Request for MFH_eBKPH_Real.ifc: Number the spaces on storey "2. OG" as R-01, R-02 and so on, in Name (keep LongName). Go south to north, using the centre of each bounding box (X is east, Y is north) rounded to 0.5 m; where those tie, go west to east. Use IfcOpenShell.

First a look at what the model holds.

```python
import ifcopenshell
import ifcopenshell.util.element
import ifcopenshell.util.placement

model = ifcopenshell.open("MFH_eBKPH_Real.ifc")
print(model.schema)
storey = next(s for s in model.by_type("IfcBuildingStorey") if s.Name == "2. OG")
spaces = [e for e in ifcopenshell.util.element.get_decomposition(storey) if e.is_a("IfcSpace")]
for e in sorted(spaces, key=lambda e: e.id()):
    origin = ifcopenshell.util.placement.get_local_placement(e.ObjectPlacement)[:3, 3]
    print(e.id(), e.Name, e.LongName, origin.round(2) + 0.0, sep=" | ")
```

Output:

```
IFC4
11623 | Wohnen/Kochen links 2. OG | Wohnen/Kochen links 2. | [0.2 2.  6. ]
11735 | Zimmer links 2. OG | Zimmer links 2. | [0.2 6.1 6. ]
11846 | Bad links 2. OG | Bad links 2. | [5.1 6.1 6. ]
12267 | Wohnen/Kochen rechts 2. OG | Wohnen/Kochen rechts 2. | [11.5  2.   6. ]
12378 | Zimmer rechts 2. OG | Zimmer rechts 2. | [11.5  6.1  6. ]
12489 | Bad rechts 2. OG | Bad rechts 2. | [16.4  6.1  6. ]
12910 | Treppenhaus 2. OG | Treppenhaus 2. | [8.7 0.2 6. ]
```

```python
import ifcopenshell
import ifcopenshell.geom
import ifcopenshell.util.element
import ifcopenshell.util.shape

model = ifcopenshell.open("MFH_eBKPH_Real.ifc")
settings = ifcopenshell.geom.settings()
settings.set("use-world-coords", True)


def centre(element):
    shape = ifcopenshell.geom.create_shape(settings, element)
    return ifcopenshell.util.shape.get_bbox_centroid(shape.geometry)


storey = next(s for s in model.by_type("IfcBuildingStorey") if s.Name == "2. OG")
spaces = [e for e in ifcopenshell.util.element.get_decomposition(storey) if e.is_a("IfcSpace")]

# Insertion points can sit at a corner or the storey origin, so sort by the geometry (in metres).
centres = {e: centre(e) for e in spaces}
spaces.sort(key=lambda e: (round(centres[e][1] / 0.5), centres[e][0]))

for i, e in enumerate(spaces, start=1):
    number = f"R-{i:02d}"
    e.Name = number
    print(e.id(), number)

model.write("MFH_eBKPH_Real-out.ifc")
```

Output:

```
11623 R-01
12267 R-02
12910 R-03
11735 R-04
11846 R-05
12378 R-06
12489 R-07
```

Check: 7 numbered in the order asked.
